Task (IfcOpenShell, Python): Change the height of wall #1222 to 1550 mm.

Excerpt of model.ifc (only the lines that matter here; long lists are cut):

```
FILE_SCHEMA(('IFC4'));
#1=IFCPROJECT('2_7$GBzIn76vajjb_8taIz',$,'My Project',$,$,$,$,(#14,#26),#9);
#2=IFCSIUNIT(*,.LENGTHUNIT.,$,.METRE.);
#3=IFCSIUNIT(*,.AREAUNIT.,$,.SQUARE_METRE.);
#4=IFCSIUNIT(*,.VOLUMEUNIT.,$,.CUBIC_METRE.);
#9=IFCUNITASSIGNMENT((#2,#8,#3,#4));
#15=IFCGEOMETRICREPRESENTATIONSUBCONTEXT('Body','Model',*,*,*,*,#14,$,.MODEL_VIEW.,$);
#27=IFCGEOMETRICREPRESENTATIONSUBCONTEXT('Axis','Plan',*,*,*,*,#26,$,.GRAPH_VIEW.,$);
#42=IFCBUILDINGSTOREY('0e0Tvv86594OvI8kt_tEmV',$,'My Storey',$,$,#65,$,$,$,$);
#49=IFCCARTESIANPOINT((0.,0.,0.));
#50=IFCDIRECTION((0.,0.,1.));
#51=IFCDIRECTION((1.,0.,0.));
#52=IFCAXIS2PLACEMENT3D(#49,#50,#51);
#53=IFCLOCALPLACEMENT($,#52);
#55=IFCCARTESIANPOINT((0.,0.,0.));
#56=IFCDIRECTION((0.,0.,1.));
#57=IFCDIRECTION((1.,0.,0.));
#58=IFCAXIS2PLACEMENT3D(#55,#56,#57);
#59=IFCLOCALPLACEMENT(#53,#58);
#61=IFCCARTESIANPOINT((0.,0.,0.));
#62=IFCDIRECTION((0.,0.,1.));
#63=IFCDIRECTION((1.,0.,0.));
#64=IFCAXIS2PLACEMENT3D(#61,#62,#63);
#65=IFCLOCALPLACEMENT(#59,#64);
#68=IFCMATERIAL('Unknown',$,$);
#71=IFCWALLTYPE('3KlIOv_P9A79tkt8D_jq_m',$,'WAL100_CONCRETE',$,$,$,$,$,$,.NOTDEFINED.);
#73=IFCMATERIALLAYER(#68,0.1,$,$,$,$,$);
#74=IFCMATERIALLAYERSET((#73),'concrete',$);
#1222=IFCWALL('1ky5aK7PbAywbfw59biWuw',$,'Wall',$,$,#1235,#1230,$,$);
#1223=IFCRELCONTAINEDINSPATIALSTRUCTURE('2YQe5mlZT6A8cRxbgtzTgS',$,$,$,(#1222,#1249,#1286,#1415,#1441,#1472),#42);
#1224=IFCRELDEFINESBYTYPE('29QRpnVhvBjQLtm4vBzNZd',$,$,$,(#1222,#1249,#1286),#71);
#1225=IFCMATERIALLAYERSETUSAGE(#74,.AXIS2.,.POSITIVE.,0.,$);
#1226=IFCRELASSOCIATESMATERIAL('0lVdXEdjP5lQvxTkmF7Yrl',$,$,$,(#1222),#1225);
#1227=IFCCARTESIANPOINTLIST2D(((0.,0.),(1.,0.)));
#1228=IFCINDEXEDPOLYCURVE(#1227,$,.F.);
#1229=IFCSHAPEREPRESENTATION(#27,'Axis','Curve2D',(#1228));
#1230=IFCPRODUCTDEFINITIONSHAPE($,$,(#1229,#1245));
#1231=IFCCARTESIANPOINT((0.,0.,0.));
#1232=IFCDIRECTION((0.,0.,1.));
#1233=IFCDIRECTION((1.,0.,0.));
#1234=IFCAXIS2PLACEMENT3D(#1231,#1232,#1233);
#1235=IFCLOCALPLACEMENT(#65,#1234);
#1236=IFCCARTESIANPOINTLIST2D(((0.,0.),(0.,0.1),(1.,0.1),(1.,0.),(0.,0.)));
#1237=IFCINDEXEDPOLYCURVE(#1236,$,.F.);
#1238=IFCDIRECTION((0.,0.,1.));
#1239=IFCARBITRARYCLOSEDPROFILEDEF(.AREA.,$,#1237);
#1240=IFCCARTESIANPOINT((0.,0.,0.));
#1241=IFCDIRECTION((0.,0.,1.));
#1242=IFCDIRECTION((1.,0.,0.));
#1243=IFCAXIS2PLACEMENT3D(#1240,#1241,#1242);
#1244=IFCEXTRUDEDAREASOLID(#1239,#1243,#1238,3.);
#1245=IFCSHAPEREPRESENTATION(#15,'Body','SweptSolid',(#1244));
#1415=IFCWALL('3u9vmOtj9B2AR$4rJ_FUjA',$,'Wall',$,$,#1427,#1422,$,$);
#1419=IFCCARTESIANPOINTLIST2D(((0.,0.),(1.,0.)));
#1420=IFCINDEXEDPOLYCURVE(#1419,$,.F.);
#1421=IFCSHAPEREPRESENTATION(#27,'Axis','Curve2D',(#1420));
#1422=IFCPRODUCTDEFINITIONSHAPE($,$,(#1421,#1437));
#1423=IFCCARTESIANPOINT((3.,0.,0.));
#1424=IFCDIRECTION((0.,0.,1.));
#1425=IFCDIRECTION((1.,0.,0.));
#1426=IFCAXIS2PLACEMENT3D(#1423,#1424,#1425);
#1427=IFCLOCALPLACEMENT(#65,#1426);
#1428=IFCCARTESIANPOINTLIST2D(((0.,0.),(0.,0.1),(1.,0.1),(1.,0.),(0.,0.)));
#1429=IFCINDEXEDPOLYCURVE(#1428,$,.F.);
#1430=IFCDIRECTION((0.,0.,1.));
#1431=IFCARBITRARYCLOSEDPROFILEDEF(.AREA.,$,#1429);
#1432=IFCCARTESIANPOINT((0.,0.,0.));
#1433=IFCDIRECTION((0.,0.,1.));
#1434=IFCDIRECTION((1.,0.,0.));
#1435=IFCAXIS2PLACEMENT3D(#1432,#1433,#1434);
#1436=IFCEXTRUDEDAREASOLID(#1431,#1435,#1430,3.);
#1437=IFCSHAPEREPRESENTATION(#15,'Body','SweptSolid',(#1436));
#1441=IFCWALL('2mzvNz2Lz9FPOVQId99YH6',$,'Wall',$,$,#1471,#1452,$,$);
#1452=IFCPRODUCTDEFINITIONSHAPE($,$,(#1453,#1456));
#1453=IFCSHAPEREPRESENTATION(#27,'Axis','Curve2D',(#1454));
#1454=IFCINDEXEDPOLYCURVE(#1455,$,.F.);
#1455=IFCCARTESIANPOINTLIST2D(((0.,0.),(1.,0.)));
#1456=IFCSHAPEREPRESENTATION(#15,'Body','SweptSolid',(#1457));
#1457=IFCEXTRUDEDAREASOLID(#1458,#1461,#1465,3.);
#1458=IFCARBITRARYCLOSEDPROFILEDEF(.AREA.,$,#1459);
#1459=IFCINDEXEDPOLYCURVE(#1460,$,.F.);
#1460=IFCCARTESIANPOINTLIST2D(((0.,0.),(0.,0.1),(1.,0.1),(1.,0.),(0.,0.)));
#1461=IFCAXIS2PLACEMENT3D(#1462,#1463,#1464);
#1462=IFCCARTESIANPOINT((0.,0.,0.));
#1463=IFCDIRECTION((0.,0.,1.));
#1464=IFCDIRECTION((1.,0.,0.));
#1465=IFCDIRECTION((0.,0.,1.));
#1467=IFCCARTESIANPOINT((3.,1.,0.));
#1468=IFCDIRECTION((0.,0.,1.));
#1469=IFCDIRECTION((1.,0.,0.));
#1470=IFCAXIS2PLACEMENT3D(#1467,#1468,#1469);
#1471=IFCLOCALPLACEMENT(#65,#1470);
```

```python
import ifcopenshell
import ifcopenshell.geom
import ifcopenshell.util.representation
import ifcopenshell.util.shape
import ifcopenshell.util.unit

model = ifcopenshell.open("model.ifc")
unit_scale = ifcopenshell.util.unit.calculate_unit_scale(model)
settings = ifcopenshell.geom.settings()


def volume(element):
    """Net volume in cubic metres, openings subtracted."""
    shape = ifcopenshell.geom.create_shape(settings, element)
    return ifcopenshell.util.shape.get_volume(shape.geometry)


wall = model.by_guid("1ky5aK7PbAywbfw59biWuw")
before = volume(wall)

body = ifcopenshell.util.representation.get_representation(wall, "Model", "Body")
solid = body.Items[0]
old_height = solid.Depth
solid.Depth = 1.55 / unit_scale
after = volume(wall)

print(f"height {old_height:g} -> {solid.Depth:g}, volume {before:.3f} -> {after:.3f} m3")

model.write("model_edited.ifc")
```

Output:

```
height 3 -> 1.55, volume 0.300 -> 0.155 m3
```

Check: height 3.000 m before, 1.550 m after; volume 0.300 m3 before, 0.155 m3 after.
